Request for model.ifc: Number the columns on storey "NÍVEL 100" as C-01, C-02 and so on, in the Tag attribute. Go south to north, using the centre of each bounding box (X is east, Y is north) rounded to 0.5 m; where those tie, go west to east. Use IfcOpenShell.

First a look at what the model holds.

```python
import ifcopenshell
import ifcopenshell.util.element
import ifcopenshell.util.placement

model = ifcopenshell.open("model.ifc")
print(model.schema)
storey = next(s for s in model.by_type("IfcBuildingStorey") if s.Name == "NÍVEL 100")
columns = [e for e in ifcopenshell.util.element.get_decomposition(storey) if e.is_a("IfcColumn")]
for e in sorted(columns, key=lambda e: e.id()):
    origin = ifcopenshell.util.placement.get_local_placement(e.ObjectPlacement)[:3, 3]
    print(e.id(), e.Tag, e.Name, origin.round(2) + 0.0, sep=" | ")
```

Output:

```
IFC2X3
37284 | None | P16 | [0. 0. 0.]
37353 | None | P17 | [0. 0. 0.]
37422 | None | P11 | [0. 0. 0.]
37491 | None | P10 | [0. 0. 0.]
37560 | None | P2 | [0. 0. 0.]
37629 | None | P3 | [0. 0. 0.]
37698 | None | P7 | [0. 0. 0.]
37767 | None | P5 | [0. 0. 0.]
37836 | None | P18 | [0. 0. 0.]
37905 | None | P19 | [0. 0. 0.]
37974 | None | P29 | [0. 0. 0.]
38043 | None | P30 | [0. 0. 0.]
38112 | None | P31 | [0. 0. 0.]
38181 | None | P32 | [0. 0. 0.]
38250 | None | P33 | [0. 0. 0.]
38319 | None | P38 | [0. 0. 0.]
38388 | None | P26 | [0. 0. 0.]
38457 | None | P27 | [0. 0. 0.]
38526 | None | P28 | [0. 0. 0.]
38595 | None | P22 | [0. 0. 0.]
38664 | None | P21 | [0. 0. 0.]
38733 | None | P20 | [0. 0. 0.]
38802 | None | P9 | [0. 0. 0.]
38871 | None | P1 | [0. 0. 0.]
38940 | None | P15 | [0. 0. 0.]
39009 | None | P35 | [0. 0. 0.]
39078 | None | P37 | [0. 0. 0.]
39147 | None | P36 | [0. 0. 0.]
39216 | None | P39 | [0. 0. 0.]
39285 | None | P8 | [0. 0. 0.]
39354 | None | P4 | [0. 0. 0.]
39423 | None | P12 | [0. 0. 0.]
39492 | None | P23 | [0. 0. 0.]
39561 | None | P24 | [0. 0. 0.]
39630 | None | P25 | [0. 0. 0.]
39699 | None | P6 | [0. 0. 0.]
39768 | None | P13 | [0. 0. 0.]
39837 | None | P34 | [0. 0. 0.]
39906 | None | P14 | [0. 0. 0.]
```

```python
import ifcopenshell
import ifcopenshell.geom
import ifcopenshell.util.element
import ifcopenshell.util.shape

model = ifcopenshell.open("model.ifc")
settings = ifcopenshell.geom.settings()
settings.set("use-world-coords", True)


def centre(element):
    shape = ifcopenshell.geom.create_shape(settings, element)
    return ifcopenshell.util.shape.get_bbox_centroid(shape.geometry)


storey = next(s for s in model.by_type("IfcBuildingStorey") if s.Name == "NÍVEL 100")
columns = [e for e in ifcopenshell.util.element.get_decomposition(storey) if e.is_a("IfcColumn")]

# Insertion points can sit at a corner or the storey origin, so sort by the geometry (in metres).
centres = {e: centre(e) for e in columns}
columns.sort(key=lambda e: (round(centres[e][1] / 0.5), centres[e][0]))

for i, e in enumerate(columns, start=1):
    number = f"C-{i:02d}"
    e.Tag = number
    print(e.id(), number)

model.write("model-out.ifc")
```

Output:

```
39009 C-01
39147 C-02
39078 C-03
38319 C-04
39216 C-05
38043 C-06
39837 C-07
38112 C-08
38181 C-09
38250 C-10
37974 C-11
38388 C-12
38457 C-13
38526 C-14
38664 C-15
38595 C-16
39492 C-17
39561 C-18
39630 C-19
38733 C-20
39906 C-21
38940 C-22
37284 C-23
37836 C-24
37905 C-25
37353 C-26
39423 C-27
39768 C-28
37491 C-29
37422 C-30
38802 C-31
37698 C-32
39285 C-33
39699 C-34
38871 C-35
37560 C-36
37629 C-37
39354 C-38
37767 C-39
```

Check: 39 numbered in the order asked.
